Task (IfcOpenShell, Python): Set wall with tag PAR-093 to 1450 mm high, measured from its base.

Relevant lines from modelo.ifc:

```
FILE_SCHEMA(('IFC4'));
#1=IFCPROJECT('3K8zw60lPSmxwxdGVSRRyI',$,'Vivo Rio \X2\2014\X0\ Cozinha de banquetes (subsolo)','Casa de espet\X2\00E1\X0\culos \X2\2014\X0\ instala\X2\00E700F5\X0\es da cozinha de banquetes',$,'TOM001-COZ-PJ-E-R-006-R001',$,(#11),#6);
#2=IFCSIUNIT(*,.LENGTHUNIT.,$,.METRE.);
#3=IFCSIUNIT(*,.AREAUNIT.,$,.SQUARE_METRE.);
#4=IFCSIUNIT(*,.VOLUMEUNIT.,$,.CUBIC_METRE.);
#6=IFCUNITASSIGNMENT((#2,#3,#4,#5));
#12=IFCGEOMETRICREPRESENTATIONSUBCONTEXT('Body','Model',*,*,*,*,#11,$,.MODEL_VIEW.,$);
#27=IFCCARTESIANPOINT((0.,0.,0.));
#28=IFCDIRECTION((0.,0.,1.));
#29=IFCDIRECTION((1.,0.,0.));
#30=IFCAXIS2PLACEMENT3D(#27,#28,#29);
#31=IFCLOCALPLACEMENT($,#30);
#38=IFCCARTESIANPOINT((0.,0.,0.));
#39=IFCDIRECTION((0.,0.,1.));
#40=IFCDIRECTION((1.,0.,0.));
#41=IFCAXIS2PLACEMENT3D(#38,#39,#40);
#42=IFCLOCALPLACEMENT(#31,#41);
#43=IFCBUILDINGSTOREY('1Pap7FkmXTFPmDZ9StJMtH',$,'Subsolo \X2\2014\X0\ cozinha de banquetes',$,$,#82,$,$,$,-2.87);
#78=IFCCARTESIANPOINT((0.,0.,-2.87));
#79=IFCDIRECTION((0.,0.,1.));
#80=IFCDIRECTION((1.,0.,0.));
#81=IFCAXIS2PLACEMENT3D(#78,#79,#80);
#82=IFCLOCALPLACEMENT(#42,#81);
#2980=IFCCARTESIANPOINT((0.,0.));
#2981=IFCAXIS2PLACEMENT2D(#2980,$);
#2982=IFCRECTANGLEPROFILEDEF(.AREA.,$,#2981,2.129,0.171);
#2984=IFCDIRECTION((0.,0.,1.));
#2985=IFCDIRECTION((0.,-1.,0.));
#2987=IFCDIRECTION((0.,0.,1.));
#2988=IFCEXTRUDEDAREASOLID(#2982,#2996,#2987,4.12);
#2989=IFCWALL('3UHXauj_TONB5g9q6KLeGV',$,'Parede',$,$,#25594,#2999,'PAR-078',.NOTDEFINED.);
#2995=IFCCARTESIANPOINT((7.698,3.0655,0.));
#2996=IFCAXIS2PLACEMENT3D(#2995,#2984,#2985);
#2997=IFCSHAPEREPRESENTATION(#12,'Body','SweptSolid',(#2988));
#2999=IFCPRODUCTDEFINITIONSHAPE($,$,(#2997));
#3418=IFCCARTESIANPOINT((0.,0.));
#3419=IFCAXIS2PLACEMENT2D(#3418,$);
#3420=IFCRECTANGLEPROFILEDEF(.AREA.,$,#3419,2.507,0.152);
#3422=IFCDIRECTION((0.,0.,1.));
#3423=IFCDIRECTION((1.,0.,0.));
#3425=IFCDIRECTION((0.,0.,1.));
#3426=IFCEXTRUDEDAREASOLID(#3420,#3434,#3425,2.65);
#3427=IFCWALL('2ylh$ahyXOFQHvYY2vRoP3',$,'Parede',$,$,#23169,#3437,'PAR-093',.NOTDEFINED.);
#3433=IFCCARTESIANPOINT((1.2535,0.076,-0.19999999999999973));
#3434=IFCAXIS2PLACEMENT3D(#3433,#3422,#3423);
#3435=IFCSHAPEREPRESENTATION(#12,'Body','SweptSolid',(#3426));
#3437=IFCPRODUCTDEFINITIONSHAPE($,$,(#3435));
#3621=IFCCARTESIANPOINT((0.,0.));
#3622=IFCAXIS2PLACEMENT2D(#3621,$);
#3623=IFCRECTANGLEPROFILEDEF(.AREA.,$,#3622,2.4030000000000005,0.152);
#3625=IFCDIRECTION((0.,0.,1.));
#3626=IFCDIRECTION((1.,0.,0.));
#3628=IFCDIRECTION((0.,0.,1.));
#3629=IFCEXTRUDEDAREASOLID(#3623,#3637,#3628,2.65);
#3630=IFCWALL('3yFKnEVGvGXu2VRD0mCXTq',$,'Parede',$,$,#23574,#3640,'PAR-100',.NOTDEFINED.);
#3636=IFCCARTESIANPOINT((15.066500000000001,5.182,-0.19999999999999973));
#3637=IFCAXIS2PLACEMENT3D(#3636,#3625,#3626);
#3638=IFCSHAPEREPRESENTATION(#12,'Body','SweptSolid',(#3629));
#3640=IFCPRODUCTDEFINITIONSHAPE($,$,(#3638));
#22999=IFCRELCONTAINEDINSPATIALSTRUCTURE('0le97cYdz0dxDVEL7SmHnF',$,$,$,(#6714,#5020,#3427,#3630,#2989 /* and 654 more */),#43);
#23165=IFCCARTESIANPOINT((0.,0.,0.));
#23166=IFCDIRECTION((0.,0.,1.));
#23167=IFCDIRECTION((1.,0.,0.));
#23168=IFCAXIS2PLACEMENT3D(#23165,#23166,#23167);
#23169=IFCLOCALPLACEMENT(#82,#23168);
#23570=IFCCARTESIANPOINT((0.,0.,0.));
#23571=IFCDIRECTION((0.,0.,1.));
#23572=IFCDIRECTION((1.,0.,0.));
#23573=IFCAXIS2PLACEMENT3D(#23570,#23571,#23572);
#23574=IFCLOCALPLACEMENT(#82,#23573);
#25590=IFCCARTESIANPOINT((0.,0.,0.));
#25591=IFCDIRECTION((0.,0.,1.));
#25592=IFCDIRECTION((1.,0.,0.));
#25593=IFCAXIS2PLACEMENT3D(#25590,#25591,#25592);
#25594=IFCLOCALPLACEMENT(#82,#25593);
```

```python
import ifcopenshell
import ifcopenshell.geom
import ifcopenshell.util.representation
import ifcopenshell.util.shape

model = ifcopenshell.open("modelo.ifc")
settings = ifcopenshell.geom.settings()


def volume(element):
    """Net volume in cubic metres, openings subtracted."""
    shape = ifcopenshell.geom.create_shape(settings, element)
    return ifcopenshell.util.shape.get_volume(shape.geometry)


wall = model.by_id(3427)
before = volume(wall)

body = ifcopenshell.util.representation.get_representation(wall, "Model", "Body")
solid = body.Items[0]
old_height = solid.Depth
solid.Depth = 1.45
after = volume(wall)

print(f"height {old_height:g} -> {solid.Depth:g}, volume {before:.3f} -> {after:.3f} m3")

model.write("modelo-out.ifc")
```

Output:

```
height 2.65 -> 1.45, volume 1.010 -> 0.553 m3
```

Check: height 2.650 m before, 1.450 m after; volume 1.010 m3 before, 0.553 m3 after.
